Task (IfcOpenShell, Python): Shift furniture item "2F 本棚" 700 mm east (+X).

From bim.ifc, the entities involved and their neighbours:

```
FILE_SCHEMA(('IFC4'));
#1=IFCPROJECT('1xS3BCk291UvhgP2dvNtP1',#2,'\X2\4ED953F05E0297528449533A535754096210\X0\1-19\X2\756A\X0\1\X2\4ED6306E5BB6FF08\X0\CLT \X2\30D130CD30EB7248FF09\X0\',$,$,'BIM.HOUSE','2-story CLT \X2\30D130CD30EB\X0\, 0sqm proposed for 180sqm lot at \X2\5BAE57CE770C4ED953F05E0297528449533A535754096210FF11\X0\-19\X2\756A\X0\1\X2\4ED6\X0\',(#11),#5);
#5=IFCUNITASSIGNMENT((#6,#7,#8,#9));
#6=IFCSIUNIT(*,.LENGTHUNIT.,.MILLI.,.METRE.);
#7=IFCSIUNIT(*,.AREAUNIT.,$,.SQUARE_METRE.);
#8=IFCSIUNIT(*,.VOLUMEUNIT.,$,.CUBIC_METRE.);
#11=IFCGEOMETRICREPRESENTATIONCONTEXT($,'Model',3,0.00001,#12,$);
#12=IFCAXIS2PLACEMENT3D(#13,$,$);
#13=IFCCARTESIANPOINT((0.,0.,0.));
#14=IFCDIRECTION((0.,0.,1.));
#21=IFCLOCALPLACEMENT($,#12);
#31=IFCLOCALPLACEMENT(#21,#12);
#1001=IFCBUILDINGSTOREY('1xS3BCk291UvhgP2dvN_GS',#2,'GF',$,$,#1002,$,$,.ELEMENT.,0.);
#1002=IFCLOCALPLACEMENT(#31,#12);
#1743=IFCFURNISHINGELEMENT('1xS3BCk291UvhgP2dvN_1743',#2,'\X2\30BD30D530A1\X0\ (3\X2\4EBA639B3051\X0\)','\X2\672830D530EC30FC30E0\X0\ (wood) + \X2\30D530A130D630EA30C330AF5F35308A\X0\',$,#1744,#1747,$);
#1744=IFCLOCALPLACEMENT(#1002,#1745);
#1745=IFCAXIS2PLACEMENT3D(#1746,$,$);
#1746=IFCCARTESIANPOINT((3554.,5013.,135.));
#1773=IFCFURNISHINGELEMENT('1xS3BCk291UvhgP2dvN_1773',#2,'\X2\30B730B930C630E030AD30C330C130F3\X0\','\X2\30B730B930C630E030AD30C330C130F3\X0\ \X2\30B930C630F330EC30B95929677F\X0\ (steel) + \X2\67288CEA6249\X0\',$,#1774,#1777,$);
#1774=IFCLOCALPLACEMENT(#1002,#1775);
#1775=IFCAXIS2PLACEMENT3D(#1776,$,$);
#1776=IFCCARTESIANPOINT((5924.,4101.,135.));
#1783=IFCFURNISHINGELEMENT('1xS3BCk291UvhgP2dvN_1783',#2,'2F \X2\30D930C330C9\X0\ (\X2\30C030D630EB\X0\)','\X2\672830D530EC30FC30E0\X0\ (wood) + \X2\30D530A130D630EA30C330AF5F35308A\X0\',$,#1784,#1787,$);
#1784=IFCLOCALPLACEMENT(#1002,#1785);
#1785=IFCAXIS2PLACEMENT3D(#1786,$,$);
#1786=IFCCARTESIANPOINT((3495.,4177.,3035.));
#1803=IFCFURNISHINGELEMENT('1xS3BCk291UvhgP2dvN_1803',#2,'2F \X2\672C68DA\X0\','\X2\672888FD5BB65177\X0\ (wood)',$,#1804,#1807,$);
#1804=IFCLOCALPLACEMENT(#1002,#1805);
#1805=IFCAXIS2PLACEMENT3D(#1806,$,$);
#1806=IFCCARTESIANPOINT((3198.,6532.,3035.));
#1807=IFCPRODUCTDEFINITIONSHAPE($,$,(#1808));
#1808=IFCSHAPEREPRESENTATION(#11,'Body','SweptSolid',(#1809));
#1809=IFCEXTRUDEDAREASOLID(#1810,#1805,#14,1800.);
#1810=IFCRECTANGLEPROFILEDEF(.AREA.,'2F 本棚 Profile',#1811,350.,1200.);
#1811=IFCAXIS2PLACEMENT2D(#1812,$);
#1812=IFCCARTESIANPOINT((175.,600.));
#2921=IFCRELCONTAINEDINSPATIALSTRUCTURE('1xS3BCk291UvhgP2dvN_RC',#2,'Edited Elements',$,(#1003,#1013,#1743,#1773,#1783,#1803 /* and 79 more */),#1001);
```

```python
import ifcopenshell
import ifcopenshell.api.geometry
import ifcopenshell.util.placement

model = ifcopenshell.open("bim.ifc")

item = model.by_id(1803)
matrix = ifcopenshell.util.placement.get_local_placement(item.ObjectPlacement)
matrix[0, 3] += 700.0
ifcopenshell.api.geometry.edit_object_placement(model, product=item, matrix=matrix, is_si=False)

print(ifcopenshell.util.placement.get_local_placement(item.ObjectPlacement).round(3) + 0.0)

model.write("bim_v2.ifc")
```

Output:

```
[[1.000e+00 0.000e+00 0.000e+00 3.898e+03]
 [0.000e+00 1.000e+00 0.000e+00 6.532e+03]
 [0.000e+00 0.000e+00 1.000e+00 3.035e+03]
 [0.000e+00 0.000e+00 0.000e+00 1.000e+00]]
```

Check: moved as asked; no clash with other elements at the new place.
